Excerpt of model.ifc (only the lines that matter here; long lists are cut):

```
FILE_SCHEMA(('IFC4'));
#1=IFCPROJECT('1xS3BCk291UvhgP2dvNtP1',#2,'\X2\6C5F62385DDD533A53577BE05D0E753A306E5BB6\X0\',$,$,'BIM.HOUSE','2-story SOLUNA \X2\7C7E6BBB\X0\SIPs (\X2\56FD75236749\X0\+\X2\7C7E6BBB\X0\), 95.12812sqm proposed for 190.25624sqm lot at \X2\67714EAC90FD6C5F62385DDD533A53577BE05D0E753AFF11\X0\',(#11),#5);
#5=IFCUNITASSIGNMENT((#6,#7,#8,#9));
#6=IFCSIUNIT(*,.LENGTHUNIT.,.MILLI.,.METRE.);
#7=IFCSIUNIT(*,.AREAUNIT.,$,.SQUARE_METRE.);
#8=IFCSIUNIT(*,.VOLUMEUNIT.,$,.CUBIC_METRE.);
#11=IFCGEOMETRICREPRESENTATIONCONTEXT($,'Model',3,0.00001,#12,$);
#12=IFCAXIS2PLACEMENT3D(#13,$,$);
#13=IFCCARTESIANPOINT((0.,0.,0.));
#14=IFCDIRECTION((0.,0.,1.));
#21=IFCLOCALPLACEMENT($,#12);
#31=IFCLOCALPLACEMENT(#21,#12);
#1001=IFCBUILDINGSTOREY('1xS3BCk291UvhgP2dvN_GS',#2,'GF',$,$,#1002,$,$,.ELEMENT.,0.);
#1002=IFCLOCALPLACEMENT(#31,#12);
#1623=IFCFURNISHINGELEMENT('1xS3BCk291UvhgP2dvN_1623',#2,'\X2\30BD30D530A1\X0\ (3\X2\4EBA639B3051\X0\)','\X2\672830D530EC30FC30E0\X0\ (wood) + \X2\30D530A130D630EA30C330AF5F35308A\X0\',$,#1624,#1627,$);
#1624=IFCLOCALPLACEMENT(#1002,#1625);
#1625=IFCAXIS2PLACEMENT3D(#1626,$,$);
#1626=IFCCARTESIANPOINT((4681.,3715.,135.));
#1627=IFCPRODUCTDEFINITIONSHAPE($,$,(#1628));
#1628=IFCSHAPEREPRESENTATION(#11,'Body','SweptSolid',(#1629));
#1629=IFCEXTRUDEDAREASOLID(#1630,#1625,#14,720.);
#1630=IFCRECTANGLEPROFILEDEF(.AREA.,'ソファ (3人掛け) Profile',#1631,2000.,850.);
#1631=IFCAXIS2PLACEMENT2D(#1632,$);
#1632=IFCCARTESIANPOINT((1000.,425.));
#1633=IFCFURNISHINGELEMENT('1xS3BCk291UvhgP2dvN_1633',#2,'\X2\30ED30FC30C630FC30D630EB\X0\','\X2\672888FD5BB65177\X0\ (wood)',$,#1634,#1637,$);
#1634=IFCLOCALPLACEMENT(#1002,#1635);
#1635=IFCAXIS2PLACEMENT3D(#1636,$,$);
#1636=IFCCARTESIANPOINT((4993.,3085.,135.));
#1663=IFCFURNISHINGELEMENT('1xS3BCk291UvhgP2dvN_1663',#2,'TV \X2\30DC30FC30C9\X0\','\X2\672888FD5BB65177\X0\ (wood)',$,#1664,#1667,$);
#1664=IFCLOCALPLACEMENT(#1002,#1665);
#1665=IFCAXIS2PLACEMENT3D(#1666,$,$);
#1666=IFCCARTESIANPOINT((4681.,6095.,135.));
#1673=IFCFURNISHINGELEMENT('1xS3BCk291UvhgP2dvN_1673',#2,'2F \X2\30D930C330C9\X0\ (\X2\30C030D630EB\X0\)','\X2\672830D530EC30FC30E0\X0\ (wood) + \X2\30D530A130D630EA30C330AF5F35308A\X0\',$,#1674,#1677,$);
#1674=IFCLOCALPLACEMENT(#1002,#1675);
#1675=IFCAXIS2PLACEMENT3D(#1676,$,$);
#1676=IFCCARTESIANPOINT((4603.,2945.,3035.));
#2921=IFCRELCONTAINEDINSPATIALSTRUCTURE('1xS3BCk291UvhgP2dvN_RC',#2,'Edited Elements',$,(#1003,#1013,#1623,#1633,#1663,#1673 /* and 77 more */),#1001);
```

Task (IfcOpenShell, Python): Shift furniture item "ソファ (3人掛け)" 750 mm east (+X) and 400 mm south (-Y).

```python
import ifcopenshell
import ifcopenshell.api.geometry
import ifcopenshell.util.placement
import ifcopenshell.util.unit

model = ifcopenshell.open("model.ifc")
unit_scale = ifcopenshell.util.unit.calculate_unit_scale(model)

item = model.by_guid("1xS3BCk291UvhgP2dvN_1623")
matrix = ifcopenshell.util.placement.get_local_placement(item.ObjectPlacement)
matrix[0, 3] += 0.75 / unit_scale
matrix[1, 3] -= 0.4 / unit_scale
ifcopenshell.api.geometry.edit_object_placement(model, product=item, matrix=matrix, is_si=False)

print(ifcopenshell.util.placement.get_local_placement(item.ObjectPlacement).round(3) + 0.0)

model.write("model_rev.ifc")
```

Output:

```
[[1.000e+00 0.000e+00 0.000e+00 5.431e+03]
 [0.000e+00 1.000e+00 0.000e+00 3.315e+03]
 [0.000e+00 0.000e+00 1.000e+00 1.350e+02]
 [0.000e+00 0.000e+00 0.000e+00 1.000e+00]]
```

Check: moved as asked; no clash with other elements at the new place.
